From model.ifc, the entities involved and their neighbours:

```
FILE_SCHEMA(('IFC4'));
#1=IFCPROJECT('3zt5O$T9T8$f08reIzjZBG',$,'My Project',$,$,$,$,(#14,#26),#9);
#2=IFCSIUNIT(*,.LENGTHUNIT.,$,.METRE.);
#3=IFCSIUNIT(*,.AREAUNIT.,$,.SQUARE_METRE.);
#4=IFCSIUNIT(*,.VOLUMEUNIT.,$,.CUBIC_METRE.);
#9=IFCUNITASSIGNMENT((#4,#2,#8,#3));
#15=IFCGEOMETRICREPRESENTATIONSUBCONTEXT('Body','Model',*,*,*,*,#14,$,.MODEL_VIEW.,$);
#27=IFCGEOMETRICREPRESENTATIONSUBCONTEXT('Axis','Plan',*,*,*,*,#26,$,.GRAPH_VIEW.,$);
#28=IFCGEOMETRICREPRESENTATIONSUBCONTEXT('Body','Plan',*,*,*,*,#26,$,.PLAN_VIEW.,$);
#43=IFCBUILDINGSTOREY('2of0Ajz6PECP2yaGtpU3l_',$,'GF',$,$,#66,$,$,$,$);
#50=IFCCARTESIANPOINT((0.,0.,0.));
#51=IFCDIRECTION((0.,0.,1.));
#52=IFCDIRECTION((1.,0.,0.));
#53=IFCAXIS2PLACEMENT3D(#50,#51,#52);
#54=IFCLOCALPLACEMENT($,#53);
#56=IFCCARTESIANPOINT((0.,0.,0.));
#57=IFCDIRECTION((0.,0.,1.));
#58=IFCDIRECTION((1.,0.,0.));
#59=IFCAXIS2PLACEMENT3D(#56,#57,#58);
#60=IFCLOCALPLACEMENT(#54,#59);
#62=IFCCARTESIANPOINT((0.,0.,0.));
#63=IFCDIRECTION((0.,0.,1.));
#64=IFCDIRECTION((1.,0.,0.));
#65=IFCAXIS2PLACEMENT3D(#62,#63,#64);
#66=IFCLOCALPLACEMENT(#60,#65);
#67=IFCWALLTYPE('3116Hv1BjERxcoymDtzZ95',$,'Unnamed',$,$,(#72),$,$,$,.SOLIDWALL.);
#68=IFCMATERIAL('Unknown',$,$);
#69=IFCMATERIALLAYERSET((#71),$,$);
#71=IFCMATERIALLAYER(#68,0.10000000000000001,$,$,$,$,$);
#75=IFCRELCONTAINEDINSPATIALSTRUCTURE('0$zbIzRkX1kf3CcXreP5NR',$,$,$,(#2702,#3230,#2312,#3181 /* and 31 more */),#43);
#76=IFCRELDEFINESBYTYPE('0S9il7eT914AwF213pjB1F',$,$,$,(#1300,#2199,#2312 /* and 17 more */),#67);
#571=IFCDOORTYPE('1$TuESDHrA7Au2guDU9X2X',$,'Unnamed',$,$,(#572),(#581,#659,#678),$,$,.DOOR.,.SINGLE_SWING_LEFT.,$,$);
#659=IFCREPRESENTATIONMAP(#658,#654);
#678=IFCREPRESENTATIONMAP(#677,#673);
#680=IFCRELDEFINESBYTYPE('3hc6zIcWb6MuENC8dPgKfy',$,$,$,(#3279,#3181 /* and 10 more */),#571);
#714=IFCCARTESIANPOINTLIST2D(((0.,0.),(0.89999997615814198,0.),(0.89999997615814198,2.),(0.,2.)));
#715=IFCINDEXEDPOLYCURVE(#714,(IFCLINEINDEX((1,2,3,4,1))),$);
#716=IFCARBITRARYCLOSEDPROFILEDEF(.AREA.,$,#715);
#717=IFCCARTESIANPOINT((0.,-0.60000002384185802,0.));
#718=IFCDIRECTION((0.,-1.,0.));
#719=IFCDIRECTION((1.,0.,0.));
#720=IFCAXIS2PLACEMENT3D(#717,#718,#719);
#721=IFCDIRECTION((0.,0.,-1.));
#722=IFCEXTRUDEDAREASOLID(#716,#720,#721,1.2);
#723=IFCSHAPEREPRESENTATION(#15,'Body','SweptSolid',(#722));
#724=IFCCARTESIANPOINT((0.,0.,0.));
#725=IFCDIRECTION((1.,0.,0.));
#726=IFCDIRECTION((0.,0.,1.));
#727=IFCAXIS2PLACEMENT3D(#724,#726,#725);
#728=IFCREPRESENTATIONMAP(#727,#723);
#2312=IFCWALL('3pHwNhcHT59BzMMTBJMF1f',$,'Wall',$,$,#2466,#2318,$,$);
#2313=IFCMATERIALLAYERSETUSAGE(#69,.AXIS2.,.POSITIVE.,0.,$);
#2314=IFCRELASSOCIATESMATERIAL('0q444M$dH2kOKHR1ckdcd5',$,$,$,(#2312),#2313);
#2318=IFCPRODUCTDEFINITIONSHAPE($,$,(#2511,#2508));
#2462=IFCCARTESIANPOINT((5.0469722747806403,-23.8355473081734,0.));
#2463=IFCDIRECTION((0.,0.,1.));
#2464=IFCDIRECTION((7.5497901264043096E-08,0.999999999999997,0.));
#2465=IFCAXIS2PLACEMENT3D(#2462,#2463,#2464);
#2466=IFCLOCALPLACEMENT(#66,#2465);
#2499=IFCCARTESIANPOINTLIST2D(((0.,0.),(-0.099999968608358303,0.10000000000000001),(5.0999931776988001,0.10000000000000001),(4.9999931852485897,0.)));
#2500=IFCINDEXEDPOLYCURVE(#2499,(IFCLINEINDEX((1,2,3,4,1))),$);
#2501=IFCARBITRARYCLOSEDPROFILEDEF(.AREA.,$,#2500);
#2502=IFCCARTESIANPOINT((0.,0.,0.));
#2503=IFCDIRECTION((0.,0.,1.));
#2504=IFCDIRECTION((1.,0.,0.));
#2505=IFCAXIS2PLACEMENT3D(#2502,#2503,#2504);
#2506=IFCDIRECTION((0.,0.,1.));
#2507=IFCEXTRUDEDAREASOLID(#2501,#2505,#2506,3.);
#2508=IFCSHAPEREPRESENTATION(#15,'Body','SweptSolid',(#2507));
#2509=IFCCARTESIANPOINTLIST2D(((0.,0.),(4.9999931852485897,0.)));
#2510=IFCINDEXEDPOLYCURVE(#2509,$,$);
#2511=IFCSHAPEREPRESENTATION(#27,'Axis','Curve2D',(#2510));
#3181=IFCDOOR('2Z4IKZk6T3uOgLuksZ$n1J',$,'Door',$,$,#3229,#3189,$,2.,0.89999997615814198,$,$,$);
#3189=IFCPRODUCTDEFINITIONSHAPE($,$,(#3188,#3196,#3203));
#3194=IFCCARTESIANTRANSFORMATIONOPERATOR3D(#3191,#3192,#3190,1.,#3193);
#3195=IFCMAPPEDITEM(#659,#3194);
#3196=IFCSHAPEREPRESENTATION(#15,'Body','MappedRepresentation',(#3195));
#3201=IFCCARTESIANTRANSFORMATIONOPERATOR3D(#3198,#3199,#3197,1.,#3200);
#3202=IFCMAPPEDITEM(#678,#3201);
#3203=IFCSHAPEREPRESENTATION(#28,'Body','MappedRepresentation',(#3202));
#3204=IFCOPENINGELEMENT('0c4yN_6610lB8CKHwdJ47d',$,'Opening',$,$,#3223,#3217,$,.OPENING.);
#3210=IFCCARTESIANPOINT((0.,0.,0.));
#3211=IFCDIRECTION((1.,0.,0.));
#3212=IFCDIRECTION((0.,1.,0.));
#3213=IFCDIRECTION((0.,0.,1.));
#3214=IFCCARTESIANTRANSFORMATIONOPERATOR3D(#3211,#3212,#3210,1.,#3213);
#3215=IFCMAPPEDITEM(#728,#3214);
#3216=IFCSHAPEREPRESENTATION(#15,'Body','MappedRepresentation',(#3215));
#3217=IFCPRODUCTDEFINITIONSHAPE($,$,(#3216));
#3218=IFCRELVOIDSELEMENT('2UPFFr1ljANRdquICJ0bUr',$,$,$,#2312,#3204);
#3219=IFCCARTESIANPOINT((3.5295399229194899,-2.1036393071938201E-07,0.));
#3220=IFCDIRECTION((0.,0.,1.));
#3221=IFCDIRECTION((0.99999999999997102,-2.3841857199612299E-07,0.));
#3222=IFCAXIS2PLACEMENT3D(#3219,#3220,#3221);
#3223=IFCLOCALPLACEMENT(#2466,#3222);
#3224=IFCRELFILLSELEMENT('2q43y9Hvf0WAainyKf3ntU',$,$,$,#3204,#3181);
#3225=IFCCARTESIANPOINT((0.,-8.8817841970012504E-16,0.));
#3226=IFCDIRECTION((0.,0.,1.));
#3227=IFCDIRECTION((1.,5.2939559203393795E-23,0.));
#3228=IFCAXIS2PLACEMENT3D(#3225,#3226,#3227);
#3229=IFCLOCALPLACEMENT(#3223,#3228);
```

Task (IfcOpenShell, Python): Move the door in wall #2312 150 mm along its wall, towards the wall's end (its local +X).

```python
import ifcopenshell
import ifcopenshell.api.geometry
import ifcopenshell.util.placement
import ifcopenshell.util.unit

model = ifcopenshell.open("model.ifc")
unit_scale = ifcopenshell.util.unit.calculate_unit_scale(model)

door = model.by_guid("2Z4IKZk6T3uOgLuksZ$n1J")
opening = door.FillsVoids[0].RelatingOpeningElement
wall = opening.VoidsElements[0].RelatingBuildingElement

wall_matrix = ifcopenshell.util.placement.get_local_placement(wall.ObjectPlacement)
shift = wall_matrix[:3, 0] * 0.15 / unit_scale
before = ifcopenshell.util.placement.get_local_placement(door.ObjectPlacement)[:3, 3].copy()

# The door is placed relative to its opening, so it follows when the opening moves.
matrix = ifcopenshell.util.placement.get_local_placement(opening.ObjectPlacement)
matrix[:3, 3] += shift
ifcopenshell.api.geometry.edit_object_placement(
    model, product=opening, matrix=matrix, is_si=False, should_transform_children=True
)

after = ifcopenshell.util.placement.get_local_placement(door.ObjectPlacement)[:3, 3]
print("door moved by", (after - before).round(3) + 0.0)

model.write("model_updated.ifc")
```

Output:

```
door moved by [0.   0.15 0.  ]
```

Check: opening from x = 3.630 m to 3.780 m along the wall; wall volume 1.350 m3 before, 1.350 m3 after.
